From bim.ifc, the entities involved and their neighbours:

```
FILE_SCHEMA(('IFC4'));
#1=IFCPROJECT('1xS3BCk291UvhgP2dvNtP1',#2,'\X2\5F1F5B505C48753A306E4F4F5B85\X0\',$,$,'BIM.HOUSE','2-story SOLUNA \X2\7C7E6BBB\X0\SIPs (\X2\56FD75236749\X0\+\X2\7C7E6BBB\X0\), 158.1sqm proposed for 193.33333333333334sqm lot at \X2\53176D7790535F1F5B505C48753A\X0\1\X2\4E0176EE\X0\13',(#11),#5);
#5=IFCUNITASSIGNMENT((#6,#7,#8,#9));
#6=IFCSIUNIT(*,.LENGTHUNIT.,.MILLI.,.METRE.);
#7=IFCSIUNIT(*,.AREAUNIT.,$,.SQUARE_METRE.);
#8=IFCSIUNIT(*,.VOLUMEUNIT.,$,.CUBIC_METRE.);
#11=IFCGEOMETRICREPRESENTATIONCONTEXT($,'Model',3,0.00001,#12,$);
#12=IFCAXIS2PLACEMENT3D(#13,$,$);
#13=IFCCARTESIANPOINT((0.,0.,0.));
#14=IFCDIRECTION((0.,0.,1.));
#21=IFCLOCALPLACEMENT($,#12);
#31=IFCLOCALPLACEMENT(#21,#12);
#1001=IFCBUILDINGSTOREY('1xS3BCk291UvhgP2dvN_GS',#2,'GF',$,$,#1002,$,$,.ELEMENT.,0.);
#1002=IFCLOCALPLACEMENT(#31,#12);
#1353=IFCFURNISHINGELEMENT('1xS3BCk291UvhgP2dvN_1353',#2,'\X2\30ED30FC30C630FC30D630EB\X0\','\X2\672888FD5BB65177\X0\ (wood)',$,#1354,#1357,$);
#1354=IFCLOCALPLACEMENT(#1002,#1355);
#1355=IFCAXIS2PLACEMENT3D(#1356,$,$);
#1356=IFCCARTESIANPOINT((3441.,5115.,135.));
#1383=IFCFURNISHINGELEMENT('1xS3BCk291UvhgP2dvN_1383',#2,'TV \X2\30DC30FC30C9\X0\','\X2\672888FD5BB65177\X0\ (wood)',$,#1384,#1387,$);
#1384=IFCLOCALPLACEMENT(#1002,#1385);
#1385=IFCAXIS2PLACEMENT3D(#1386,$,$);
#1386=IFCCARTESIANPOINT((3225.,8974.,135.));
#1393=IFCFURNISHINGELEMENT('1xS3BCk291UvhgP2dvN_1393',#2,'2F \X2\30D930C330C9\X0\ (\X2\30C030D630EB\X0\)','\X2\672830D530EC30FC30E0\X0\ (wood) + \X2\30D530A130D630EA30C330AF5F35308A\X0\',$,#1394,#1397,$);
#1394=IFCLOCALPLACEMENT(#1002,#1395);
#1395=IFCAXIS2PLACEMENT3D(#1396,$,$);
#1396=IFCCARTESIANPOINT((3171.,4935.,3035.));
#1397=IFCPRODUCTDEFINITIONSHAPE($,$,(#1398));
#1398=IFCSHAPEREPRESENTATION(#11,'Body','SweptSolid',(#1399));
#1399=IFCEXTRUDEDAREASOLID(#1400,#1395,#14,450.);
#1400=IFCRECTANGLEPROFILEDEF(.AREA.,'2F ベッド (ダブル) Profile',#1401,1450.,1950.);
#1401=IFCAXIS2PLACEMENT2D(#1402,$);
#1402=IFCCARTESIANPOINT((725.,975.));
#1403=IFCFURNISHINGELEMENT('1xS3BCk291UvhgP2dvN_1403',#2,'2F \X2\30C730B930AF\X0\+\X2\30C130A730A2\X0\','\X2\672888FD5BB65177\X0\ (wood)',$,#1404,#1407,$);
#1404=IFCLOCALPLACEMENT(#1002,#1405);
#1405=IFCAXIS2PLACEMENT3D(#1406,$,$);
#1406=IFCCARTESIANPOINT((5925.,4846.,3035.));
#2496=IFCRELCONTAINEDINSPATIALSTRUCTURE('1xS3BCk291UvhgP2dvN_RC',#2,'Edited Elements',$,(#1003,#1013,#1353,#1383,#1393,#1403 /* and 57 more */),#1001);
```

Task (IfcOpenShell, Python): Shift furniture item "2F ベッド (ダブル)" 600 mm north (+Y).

```python
import ifcopenshell
import ifcopenshell.api.geometry
import ifcopenshell.util.placement

model = ifcopenshell.open("bim.ifc")

item = model.by_id(1393)
matrix = ifcopenshell.util.placement.get_local_placement(item.ObjectPlacement)
matrix[1, 3] += 600.0
ifcopenshell.api.geometry.edit_object_placement(model, product=item, matrix=matrix, is_si=False)

print(ifcopenshell.util.placement.get_local_placement(item.ObjectPlacement).round(3) + 0.0)

model.write("bim_updated.ifc")
```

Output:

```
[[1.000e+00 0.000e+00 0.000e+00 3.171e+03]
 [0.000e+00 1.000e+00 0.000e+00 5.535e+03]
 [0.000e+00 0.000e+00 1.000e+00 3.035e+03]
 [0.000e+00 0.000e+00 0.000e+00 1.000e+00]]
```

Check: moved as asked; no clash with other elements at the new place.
